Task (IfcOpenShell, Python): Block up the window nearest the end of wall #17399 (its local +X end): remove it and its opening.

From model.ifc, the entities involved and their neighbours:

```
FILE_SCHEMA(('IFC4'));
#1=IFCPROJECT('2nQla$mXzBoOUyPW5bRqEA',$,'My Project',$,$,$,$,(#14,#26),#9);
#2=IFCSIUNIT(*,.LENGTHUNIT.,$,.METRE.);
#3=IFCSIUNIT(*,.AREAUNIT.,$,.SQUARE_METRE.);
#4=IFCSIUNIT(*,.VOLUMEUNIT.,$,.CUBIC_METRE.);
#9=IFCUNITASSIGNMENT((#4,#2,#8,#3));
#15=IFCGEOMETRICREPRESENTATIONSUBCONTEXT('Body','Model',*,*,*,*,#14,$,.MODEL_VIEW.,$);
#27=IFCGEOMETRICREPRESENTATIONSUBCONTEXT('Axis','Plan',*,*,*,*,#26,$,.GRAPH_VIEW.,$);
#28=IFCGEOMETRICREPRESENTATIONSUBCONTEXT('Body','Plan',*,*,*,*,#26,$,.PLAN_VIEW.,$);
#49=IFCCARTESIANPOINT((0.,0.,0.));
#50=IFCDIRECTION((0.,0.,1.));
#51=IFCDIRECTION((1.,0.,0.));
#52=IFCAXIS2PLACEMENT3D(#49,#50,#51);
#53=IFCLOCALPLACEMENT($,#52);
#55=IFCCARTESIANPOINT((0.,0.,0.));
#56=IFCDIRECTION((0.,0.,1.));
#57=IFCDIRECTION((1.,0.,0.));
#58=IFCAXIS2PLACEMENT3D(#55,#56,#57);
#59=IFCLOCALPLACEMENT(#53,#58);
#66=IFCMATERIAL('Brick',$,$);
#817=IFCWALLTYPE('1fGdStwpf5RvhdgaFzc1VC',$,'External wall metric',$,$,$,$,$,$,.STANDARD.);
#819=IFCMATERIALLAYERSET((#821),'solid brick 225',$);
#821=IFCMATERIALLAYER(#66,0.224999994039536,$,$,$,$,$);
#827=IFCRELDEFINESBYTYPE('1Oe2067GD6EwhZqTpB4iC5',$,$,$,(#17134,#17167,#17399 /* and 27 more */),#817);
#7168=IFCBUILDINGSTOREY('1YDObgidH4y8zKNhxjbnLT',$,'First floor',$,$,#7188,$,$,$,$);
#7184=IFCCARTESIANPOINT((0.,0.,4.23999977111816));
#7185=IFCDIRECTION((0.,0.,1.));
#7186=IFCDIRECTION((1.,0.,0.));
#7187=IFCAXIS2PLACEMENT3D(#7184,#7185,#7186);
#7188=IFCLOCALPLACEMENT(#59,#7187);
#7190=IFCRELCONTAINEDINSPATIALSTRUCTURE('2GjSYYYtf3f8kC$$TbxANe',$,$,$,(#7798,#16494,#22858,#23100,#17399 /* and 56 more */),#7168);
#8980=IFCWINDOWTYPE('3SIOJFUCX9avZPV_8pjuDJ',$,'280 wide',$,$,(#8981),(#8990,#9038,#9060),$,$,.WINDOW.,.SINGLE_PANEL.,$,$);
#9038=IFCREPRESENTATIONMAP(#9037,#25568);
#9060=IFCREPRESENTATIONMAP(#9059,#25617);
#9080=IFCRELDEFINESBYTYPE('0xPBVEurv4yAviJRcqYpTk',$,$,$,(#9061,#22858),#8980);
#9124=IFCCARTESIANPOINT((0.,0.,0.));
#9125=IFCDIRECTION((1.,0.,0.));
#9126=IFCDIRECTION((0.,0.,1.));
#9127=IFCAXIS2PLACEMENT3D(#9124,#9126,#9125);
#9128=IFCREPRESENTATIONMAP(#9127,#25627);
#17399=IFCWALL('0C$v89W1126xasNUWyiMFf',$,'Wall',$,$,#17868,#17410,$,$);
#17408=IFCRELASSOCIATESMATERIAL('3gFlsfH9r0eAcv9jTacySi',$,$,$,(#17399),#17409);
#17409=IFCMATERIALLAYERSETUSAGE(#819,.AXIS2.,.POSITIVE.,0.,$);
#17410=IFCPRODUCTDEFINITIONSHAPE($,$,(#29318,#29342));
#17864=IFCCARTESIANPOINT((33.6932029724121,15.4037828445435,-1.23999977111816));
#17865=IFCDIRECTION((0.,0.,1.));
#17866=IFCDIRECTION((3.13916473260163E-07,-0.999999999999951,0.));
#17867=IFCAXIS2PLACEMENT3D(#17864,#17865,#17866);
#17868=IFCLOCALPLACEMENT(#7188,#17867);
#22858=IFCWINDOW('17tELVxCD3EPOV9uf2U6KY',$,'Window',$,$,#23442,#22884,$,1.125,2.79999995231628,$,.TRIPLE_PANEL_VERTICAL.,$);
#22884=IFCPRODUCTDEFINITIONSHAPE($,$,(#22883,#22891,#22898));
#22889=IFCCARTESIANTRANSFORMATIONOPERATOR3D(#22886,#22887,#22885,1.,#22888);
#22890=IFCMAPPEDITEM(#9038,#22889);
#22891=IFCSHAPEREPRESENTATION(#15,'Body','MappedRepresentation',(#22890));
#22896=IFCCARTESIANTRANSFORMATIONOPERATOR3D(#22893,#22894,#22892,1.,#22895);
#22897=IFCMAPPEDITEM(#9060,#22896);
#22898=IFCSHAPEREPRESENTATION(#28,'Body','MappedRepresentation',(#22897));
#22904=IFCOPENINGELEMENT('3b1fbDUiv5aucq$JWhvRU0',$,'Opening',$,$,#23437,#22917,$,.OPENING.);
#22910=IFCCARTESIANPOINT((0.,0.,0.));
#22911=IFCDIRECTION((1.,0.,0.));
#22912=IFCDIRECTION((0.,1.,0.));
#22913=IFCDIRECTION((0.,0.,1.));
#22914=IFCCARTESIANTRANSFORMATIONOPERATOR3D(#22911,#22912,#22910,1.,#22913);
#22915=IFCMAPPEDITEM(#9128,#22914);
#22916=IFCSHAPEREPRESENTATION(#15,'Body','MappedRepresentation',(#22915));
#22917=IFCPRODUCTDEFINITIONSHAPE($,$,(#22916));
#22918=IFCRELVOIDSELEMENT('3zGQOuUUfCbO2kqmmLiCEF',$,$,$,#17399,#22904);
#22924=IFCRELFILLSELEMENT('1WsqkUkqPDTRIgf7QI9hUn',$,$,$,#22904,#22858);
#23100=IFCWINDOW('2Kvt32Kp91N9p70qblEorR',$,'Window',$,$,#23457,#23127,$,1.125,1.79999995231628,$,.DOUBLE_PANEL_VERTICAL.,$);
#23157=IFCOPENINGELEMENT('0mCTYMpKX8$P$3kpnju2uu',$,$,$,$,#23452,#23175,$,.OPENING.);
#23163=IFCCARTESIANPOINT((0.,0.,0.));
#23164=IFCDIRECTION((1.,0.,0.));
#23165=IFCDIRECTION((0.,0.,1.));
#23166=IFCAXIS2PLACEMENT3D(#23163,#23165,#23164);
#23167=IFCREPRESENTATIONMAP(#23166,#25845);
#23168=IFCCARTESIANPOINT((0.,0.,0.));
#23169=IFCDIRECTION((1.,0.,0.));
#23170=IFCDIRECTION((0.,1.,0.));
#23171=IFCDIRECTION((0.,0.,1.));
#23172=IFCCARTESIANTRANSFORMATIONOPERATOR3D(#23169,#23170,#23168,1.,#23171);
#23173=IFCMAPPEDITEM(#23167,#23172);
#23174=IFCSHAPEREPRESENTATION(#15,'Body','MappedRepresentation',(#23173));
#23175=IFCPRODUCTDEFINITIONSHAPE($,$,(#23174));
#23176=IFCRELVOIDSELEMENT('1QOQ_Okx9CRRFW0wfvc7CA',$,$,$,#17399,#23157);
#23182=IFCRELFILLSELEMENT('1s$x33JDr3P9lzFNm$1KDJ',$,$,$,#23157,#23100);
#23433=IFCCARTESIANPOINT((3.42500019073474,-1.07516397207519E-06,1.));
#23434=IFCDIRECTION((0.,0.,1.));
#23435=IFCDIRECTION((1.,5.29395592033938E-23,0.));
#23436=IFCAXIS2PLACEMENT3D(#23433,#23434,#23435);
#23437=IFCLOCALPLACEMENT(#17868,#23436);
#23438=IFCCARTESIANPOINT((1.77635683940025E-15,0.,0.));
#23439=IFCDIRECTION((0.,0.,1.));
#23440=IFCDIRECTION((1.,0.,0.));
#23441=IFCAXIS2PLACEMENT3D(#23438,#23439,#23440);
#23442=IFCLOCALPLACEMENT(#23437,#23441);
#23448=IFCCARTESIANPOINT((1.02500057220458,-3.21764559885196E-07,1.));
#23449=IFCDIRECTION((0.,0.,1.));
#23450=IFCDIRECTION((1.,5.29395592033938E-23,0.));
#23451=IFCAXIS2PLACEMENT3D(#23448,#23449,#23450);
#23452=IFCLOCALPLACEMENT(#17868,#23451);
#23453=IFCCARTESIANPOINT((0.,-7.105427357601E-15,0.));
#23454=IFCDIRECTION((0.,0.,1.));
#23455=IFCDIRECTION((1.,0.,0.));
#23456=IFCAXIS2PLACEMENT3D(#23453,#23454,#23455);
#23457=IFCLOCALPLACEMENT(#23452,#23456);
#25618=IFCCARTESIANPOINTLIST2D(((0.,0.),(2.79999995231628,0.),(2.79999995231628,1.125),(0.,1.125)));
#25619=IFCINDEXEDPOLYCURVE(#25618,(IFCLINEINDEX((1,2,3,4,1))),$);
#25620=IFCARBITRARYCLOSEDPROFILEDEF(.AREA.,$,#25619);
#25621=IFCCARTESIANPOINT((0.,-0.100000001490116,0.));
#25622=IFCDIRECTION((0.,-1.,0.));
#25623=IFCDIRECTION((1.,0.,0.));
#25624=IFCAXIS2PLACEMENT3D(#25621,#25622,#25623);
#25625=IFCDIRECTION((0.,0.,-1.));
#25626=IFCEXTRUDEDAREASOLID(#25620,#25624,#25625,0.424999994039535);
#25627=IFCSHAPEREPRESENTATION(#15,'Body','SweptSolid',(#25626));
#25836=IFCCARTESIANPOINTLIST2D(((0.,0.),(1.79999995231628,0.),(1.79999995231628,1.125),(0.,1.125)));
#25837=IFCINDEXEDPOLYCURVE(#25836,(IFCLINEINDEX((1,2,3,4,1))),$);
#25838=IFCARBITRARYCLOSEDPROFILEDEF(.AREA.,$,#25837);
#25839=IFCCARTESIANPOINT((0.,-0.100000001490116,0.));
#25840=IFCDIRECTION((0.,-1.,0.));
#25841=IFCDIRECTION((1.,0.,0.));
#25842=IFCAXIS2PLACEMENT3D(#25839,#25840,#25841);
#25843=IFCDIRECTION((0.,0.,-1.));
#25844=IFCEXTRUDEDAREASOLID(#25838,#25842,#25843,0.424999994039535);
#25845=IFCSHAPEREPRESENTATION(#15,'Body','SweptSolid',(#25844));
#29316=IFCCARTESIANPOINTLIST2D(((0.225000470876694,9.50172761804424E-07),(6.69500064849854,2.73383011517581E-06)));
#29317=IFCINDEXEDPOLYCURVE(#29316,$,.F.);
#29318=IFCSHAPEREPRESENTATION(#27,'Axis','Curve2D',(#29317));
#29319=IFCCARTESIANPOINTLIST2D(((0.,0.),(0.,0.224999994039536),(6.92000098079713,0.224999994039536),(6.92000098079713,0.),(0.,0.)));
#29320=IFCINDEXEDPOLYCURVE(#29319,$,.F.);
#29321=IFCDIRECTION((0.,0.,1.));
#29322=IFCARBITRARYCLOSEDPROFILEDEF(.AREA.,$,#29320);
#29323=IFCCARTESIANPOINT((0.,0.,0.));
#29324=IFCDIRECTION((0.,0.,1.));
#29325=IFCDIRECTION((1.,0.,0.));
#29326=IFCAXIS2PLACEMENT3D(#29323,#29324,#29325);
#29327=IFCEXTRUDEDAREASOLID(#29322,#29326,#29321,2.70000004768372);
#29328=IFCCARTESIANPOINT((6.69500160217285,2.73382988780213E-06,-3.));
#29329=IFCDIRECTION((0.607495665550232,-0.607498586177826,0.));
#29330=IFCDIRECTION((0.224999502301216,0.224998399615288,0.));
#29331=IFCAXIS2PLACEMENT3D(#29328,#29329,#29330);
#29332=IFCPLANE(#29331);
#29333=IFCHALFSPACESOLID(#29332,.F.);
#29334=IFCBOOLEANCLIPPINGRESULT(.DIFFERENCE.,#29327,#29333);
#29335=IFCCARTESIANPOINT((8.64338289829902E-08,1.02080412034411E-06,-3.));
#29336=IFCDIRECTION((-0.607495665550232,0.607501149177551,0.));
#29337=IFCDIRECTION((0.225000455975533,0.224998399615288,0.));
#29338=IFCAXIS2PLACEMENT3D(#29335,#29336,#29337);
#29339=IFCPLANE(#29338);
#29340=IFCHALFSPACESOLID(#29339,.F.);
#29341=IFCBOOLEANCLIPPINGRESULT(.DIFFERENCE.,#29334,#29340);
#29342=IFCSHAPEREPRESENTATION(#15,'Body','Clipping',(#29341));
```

```python
import ifcopenshell
import ifcopenshell.api.feature
import ifcopenshell.api.root
import ifcopenshell.geom
import ifcopenshell.util.shape

model = ifcopenshell.open("model.ifc")
settings = ifcopenshell.geom.settings()


def volume(element):
    """Net volume in cubic metres, openings subtracted."""
    shape = ifcopenshell.geom.create_shape(settings, element)
    return ifcopenshell.util.shape.get_volume(shape.geometry)


window = model.by_guid("17tELVxCD3EPOV9uf2U6KY")
opening = window.FillsVoids[0].RelatingOpeningElement
wall = opening.VoidsElements[0].RelatingBuildingElement
before = volume(wall)

ifcopenshell.api.root.remove_product(model, product=window)
ifcopenshell.api.feature.remove_feature(model, feature=opening)

after = volume(wall)

print(f"wall volume {before:.3f} -> {after:.3f} m3")

model.write("model-out.ifc")
```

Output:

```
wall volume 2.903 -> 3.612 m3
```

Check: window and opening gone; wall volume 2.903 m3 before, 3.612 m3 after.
